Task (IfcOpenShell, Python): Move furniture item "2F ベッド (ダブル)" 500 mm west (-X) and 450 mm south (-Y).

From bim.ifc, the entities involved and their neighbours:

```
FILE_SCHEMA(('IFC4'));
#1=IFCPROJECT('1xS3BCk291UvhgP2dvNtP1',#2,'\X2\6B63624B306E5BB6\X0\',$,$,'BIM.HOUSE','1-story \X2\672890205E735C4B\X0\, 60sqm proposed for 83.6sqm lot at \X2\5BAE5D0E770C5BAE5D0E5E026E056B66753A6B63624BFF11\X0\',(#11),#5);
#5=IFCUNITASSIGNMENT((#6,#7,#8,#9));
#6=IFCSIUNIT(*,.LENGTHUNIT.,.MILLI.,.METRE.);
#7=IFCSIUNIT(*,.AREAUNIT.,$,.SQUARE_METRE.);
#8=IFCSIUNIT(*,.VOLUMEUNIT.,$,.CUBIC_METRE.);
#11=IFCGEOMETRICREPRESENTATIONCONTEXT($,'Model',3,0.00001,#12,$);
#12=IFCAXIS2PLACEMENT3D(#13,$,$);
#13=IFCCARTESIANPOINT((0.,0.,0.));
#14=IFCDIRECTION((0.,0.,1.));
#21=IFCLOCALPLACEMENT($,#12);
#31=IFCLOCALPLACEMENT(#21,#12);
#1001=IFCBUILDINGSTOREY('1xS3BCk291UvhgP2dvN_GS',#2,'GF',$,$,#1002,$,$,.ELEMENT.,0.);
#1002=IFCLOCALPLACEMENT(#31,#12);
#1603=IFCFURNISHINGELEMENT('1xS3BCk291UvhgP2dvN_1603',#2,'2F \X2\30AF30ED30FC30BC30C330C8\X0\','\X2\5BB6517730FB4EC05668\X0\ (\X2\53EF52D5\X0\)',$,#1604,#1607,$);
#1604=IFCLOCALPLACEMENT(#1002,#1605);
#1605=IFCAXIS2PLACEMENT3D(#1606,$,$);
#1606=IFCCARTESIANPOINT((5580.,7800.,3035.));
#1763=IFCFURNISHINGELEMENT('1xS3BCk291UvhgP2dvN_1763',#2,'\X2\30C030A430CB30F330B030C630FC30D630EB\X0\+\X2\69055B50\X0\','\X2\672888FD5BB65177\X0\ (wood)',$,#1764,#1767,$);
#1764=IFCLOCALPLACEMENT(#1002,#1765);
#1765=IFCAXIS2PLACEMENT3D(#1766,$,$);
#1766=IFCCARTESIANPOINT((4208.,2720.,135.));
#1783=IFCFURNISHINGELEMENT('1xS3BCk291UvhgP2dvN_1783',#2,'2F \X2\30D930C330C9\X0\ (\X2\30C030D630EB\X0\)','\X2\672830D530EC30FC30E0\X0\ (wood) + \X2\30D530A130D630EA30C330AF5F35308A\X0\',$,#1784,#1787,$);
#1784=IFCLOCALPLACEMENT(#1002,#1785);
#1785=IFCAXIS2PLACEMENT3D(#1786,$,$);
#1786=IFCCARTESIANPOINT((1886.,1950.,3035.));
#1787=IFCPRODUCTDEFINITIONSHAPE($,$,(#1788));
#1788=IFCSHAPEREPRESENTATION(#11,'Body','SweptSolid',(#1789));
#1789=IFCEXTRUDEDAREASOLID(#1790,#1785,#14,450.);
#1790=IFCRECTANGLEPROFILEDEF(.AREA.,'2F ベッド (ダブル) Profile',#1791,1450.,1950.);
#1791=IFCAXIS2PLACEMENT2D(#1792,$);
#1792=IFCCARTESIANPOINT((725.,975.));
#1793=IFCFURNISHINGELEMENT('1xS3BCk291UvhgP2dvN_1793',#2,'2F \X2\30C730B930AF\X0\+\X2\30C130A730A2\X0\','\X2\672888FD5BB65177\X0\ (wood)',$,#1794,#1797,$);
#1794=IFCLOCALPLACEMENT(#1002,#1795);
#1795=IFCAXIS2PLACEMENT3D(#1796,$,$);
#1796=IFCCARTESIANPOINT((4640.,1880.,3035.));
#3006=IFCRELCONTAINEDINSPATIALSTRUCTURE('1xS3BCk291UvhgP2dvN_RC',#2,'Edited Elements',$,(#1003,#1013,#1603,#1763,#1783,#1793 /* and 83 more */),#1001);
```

```python
import ifcopenshell
import ifcopenshell.api.geometry
import ifcopenshell.util.placement
import ifcopenshell.util.unit

model = ifcopenshell.open("bim.ifc")
unit_scale = ifcopenshell.util.unit.calculate_unit_scale(model)

item = model.by_guid("1xS3BCk291UvhgP2dvN_1783")
matrix = ifcopenshell.util.placement.get_local_placement(item.ObjectPlacement)
matrix[0, 3] -= 0.5 / unit_scale
matrix[1, 3] -= 0.45 / unit_scale
ifcopenshell.api.geometry.edit_object_placement(model, product=item, matrix=matrix, is_si=False)

print(ifcopenshell.util.placement.get_local_placement(item.ObjectPlacement).round(3) + 0.0)

model.write("bim_updated.ifc")
```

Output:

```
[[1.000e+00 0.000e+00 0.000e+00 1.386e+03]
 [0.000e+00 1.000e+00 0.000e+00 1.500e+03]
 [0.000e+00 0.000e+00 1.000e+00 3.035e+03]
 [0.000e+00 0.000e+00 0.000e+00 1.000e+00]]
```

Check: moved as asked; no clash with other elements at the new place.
